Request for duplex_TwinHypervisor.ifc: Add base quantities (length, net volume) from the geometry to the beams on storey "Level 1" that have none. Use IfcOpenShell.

First a look at what the model holds.

```python
import ifcopenshell
import ifcopenshell.util.element
import ifcopenshell.util.unit

model = ifcopenshell.open("duplex_TwinHypervisor.ifc")
print(model.schema)
for unit_type in ("LENGTHUNIT", "AREAUNIT", "VOLUMEUNIT"):
    print(unit_type, ifcopenshell.util.unit.calculate_unit_scale(model, unit_type))
storey = next(s for s in model.by_type("IfcBuildingStorey") if s.Name == "Level 1")
beams = [e for e in ifcopenshell.util.element.get_decomposition(storey) if e.is_a("IfcBeam")]
for e in sorted(beams, key=lambda e: e.id()):
    print(e.id(), e.is_a(), e.Name, list(ifcopenshell.util.element.get_psets(e, qtos_only=True)), sep=" | ")
```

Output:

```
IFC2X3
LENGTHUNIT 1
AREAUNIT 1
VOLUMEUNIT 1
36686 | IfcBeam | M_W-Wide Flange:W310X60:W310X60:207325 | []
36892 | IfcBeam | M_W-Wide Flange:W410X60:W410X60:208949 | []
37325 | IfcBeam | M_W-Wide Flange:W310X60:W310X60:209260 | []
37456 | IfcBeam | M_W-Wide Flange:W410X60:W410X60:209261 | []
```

```python
import ifcopenshell
import ifcopenshell.api.pset
import ifcopenshell.geom
import ifcopenshell.util.element
import ifcopenshell.util.shape
import ifcopenshell.util.unit

model = ifcopenshell.open("duplex_TwinHypervisor.ifc")
unit_scale = ifcopenshell.util.unit.calculate_unit_scale(model)
volume_scale = ifcopenshell.util.unit.calculate_unit_scale(model, "VOLUMEUNIT")
settings = ifcopenshell.geom.settings()

storey = next(s for s in model.by_type("IfcBuildingStorey") if s.Name == "Level 1")
beams = [e for e in ifcopenshell.util.element.get_decomposition(storey) if e.is_a("IfcBeam")]

for e in sorted(beams, key=lambda e: e.id()):
    if ifcopenshell.util.element.get_psets(e, qtos_only=True, should_inherit=False):
        continue
    # Geometry comes back in metres, in the element's own axes.
    shape = ifcopenshell.geom.create_shape(settings, e)
    values = {
        "Length": ifcopenshell.util.shape.get_max_xyz(shape.geometry) / unit_scale,
        "NetVolume": ifcopenshell.util.shape.get_volume(shape.geometry) / volume_scale,
    }
    qto = ifcopenshell.api.pset.add_qto(model, product=e, name="BaseQuantities")
    ifcopenshell.api.pset.edit_qto(model, qto=qto, properties=values)
    print(e.id(), {k: round(v, 3) for k, v in values.items()})

model.write("duplex_TwinHypervisor_edited.ifc")
```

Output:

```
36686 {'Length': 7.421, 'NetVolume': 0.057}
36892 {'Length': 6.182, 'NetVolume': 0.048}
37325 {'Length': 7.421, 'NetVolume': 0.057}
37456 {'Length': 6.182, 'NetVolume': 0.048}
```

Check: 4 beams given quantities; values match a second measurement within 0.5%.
